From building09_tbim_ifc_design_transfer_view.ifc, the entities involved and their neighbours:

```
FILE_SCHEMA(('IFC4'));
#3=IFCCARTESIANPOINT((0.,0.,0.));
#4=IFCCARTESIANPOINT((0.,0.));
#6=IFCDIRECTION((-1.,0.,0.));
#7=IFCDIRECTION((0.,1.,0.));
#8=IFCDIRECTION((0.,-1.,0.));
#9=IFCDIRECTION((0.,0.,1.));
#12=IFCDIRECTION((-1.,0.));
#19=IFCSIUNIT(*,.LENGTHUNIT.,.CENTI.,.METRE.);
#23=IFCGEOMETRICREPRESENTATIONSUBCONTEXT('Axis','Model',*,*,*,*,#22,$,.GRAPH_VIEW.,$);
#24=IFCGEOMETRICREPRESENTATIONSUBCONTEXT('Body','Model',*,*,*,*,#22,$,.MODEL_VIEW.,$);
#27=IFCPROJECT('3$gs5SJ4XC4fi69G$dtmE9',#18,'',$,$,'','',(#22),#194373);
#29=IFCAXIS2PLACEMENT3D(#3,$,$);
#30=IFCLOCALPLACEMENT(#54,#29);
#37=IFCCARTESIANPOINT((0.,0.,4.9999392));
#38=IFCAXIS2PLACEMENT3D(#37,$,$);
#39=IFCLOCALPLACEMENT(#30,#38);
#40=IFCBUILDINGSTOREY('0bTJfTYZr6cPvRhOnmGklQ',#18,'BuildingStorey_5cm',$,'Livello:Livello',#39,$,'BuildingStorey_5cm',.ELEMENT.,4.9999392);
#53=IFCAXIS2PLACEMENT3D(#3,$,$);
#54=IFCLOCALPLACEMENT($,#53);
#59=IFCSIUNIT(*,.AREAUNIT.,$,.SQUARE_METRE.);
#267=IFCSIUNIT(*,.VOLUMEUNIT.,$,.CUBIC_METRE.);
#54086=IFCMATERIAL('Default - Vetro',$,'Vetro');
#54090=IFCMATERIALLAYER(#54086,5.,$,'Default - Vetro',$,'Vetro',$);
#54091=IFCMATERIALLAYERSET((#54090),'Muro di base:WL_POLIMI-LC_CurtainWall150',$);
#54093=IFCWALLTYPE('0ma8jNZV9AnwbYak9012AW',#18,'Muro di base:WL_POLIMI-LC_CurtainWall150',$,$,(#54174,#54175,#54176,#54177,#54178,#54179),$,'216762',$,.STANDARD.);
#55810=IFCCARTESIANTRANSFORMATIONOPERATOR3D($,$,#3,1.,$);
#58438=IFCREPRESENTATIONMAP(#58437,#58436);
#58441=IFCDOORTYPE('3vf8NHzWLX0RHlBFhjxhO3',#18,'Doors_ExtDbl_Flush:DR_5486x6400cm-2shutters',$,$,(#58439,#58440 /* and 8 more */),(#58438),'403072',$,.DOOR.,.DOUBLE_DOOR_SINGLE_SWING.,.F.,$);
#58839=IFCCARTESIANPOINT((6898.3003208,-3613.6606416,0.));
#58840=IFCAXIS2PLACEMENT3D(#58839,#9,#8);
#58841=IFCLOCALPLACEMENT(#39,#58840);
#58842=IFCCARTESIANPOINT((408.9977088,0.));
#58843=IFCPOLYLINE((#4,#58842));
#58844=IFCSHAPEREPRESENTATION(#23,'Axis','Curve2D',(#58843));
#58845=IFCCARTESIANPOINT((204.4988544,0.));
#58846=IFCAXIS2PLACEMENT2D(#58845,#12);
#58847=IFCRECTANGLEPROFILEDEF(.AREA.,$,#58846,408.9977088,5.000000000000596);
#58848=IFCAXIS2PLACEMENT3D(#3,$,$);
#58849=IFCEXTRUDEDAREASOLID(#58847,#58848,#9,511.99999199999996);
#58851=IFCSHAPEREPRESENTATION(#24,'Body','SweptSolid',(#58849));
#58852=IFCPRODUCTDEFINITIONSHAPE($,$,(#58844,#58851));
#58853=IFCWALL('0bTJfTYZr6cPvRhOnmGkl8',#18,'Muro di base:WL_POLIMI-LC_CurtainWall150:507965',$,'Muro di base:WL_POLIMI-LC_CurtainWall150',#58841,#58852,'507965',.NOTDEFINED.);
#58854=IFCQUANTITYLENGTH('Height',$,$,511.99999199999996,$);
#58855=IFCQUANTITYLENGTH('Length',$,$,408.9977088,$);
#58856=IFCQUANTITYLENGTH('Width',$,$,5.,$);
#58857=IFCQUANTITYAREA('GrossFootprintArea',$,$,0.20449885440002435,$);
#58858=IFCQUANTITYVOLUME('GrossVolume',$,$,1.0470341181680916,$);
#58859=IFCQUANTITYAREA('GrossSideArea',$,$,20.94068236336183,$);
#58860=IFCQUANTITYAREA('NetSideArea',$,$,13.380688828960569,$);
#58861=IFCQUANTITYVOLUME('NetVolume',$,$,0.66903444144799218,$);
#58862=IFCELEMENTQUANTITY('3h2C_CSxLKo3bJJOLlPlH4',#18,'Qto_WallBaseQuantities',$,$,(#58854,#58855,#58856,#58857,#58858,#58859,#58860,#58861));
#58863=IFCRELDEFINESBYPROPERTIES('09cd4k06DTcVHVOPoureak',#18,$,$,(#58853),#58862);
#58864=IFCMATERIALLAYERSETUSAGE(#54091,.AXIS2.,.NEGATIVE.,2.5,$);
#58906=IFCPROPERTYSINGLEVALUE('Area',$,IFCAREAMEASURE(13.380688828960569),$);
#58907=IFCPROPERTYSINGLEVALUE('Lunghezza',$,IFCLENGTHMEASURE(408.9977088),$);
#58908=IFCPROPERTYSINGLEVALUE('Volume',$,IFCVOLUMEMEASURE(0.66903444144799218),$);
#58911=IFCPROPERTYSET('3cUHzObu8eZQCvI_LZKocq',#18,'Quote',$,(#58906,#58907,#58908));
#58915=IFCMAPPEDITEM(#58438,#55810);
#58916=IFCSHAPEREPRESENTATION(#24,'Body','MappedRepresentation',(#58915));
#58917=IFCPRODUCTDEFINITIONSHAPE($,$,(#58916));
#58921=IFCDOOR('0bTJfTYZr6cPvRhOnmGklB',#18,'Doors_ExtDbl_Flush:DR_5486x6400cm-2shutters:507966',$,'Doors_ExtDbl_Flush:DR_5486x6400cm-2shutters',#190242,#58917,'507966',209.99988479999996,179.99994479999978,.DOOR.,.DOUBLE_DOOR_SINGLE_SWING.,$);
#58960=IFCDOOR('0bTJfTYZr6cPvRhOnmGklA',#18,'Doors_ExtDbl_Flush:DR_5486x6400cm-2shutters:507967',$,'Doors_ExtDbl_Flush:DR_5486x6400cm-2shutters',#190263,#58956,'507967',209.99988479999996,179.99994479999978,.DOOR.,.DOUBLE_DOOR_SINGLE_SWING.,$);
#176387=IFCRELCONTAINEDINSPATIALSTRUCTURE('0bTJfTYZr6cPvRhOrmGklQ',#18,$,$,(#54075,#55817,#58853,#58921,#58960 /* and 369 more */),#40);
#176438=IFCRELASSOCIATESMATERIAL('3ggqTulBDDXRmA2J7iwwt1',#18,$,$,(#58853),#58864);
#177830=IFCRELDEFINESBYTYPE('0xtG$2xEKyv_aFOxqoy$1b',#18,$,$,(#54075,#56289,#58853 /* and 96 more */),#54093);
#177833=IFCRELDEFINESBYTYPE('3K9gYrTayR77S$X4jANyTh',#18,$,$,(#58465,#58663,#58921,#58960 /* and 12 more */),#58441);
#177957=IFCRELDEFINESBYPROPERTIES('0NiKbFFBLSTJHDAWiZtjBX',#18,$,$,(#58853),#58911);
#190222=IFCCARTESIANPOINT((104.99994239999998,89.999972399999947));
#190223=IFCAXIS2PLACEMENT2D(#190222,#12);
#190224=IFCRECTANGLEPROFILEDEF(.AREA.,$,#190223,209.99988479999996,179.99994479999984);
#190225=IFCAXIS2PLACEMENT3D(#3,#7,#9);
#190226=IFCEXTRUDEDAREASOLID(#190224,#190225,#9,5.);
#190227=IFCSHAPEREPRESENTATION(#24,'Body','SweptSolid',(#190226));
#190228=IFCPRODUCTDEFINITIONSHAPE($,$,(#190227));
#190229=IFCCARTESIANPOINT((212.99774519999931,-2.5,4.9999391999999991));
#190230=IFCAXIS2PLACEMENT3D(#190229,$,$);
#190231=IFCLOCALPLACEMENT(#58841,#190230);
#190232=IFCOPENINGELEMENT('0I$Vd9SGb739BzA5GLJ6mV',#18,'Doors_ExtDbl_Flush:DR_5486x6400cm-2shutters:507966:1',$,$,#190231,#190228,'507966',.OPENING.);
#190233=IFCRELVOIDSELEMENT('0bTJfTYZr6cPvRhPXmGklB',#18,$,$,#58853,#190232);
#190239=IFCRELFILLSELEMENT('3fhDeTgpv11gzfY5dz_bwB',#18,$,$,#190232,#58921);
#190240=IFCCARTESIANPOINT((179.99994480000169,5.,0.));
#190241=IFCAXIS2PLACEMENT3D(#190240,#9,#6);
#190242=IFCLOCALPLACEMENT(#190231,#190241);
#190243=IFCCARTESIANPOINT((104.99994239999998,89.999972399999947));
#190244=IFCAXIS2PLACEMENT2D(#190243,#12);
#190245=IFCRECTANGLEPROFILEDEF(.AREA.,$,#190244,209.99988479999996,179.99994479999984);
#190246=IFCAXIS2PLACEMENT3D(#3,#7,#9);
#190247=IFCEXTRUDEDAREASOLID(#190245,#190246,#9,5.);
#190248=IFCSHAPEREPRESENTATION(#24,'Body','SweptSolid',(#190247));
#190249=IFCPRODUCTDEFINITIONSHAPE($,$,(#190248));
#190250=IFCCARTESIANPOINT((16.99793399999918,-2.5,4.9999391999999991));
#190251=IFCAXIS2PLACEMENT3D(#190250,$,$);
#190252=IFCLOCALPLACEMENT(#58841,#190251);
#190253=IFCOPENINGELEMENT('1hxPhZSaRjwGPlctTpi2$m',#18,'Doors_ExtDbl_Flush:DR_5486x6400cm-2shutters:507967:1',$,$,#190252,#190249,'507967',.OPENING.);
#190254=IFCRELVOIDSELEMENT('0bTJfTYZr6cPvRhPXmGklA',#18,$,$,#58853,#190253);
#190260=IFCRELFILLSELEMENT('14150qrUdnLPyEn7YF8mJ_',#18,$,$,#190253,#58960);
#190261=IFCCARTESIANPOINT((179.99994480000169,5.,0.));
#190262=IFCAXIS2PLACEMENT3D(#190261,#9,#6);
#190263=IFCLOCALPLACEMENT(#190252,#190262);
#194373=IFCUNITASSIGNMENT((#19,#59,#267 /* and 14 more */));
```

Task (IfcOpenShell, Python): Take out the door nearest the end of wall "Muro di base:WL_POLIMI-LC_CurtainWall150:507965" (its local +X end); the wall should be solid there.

```python
import ifcopenshell
import ifcopenshell.api.feature
import ifcopenshell.api.pset
import ifcopenshell.api.root
import ifcopenshell.geom
import ifcopenshell.util.element
import ifcopenshell.util.shape
import ifcopenshell.util.unit

model = ifcopenshell.open("building09_tbim_ifc_design_transfer_view.ifc")
area_scale = ifcopenshell.util.unit.calculate_unit_scale(model, "AREAUNIT")
volume_scale = ifcopenshell.util.unit.calculate_unit_scale(model, "VOLUMEUNIT")
settings = ifcopenshell.geom.settings()


def volume(element):
    """Net volume in cubic metres, openings subtracted."""
    shape = ifcopenshell.geom.create_shape(settings, element)
    return ifcopenshell.util.shape.get_volume(shape.geometry)


door = model.by_guid("0bTJfTYZr6cPvRhOnmGklB")
opening = door.FillsVoids[0].RelatingOpeningElement
wall = opening.VoidsElements[0].RelatingBuildingElement
before = volume(wall)

ifcopenshell.api.root.remove_product(model, product=door)
ifcopenshell.api.feature.remove_feature(model, feature=opening)

after = volume(wall)
thickness = 0.05  # wall thickness in metres

# Update the wall's stored quantities.
qto = model.by_id(ifcopenshell.util.element.get_pset(wall, "Qto_WallBaseQuantities", should_inherit=False)["id"])
ifcopenshell.api.pset.edit_qto(model, qto=qto, properties={
    "NetSideArea": after / thickness / area_scale,
    "NetVolume": after / volume_scale,
})
pset = model.by_id(ifcopenshell.util.element.get_pset(wall, "Quote", should_inherit=False)["id"])
ifcopenshell.api.pset.edit_pset(model, pset=pset, properties={
    "Area": model.create_entity("IfcAreaMeasure", after / thickness / area_scale),
    "Volume": model.create_entity("IfcVolumeMeasure", after / volume_scale),
})

print(f"wall volume {before:.3f} -> {after:.3f} m3")

model.write("building09_tbim_ifc_design_transfer_view-out.ifc")
```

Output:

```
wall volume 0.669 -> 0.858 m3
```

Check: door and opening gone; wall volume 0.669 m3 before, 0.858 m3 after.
